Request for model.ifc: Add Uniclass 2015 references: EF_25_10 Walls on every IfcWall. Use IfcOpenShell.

First a look at what the model holds.

```python
import ifcopenshell

model = ifcopenshell.open("model.ifc")
print(model.schema)
print("classifications:", [c.Name for c in model.by_type("IfcClassification")])
for ifc_class in ("IfcDoor", "IfcRoof", "IfcStair", "IfcWall", "IfcWindow"):
    print(ifc_class, len(model.by_type(ifc_class)))
```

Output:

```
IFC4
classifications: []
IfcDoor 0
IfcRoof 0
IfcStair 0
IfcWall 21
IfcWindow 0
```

```python
import ifcopenshell
import ifcopenshell.api.classification

model = ifcopenshell.open("model.ifc")

system = ifcopenshell.api.classification.add_classification(model, classification="Uniclass 2015")

codes = {
    "IfcWall": ("EF_25_10", "Walls"),
}
for ifc_class, (code, name) in codes.items():
    products = model.by_type(ifc_class)
    ifcopenshell.api.classification.add_reference(
        model, products=products, classification=system, identification=code, name=name
    )
    print(code, len(products))

model.write("model_v2.ifc")
```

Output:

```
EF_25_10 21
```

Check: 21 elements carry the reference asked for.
